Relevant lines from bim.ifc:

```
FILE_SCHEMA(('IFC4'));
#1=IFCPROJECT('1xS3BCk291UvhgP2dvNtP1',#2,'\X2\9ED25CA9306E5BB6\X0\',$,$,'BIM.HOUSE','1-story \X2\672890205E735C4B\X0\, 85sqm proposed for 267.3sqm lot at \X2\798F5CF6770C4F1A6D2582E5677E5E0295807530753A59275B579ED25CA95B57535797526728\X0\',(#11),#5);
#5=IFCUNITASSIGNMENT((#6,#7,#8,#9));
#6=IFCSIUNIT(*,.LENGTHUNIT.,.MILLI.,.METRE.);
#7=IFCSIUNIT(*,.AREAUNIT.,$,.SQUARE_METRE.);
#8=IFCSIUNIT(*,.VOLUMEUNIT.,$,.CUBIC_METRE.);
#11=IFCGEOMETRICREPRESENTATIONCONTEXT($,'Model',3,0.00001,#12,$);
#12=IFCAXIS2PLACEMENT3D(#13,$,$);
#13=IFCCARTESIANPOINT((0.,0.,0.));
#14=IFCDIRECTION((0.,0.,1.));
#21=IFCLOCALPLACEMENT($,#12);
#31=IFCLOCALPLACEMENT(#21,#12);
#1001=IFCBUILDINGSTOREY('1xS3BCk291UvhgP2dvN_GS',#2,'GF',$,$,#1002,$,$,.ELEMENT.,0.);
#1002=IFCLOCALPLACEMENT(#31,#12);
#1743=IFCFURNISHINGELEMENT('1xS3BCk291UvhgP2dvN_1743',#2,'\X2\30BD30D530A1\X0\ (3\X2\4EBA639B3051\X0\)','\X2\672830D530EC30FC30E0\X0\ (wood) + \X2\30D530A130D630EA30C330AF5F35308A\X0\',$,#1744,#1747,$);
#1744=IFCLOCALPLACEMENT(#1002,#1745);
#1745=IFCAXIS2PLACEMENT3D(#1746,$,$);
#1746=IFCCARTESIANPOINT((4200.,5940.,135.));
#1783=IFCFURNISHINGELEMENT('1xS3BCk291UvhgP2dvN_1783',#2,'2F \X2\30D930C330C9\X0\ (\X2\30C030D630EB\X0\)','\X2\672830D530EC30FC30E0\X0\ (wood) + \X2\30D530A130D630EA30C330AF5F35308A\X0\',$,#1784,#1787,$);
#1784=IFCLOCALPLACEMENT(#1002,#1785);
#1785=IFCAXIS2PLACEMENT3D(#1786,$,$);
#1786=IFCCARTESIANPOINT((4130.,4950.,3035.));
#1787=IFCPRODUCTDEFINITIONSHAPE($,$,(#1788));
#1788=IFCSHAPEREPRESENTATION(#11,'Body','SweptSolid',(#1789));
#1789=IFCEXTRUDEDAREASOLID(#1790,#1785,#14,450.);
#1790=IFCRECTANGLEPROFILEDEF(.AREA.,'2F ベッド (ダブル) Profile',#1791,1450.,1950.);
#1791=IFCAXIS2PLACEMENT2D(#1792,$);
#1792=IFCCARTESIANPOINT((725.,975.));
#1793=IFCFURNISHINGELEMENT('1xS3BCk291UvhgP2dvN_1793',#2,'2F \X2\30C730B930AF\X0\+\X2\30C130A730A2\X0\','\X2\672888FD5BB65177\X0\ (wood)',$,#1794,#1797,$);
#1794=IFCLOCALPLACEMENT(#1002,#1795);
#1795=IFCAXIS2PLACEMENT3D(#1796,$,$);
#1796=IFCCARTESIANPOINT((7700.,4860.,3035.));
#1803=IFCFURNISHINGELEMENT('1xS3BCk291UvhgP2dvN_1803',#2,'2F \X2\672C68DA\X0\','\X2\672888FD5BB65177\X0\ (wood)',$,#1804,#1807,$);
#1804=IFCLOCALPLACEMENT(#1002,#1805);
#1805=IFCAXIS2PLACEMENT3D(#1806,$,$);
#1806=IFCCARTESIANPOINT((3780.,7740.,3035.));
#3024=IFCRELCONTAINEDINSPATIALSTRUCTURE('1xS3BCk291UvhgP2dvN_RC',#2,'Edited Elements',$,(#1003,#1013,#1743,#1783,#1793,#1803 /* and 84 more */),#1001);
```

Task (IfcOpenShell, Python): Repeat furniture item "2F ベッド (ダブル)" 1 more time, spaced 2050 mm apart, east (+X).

```python
import numpy as np
import ifcopenshell
import ifcopenshell.api.geometry
import ifcopenshell.api.root
import ifcopenshell.util.element
import ifcopenshell.util.placement

model = ifcopenshell.open("bim.ifc")


def reuse_history(source, copy):
    """copy_class also copies each property set's owner history, people and application; keep the originals."""
    for rel in copy.IsDefinedBy:
        if rel.is_a("IfcRelDefinesByProperties") and (history := rel.RelatingPropertyDefinition.OwnerHistory):
            rel.RelatingPropertyDefinition.OwnerHistory = source.OwnerHistory
            ifcopenshell.util.element.remove_deep2(model, history)


source = model.by_guid("1xS3BCk291UvhgP2dvN_1783")
base = ifcopenshell.util.placement.get_local_placement(source.ObjectPlacement)
step = np.array([1.0, 0.0, 0.0]) * 2050.0

for i in range(1, 2):
    copy = ifcopenshell.api.root.copy_class(model, product=source)
    copy.Representation = ifcopenshell.util.element.copy_deep(
        model, source.Representation, exclude=["IfcGeometricRepresentationContext", "IfcRepresentationMap"]
    )
    reuse_history(source, copy)
    matrix = base.copy()
    matrix[:3, 3] += i * step
    print("added at", matrix[:3, 3].round(3) + 0.0)
    ifcopenshell.api.geometry.edit_object_placement(model, product=copy, matrix=matrix, is_si=False)

model.write("bim_v2.ifc")
```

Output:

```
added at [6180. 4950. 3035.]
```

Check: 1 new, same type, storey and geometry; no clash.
